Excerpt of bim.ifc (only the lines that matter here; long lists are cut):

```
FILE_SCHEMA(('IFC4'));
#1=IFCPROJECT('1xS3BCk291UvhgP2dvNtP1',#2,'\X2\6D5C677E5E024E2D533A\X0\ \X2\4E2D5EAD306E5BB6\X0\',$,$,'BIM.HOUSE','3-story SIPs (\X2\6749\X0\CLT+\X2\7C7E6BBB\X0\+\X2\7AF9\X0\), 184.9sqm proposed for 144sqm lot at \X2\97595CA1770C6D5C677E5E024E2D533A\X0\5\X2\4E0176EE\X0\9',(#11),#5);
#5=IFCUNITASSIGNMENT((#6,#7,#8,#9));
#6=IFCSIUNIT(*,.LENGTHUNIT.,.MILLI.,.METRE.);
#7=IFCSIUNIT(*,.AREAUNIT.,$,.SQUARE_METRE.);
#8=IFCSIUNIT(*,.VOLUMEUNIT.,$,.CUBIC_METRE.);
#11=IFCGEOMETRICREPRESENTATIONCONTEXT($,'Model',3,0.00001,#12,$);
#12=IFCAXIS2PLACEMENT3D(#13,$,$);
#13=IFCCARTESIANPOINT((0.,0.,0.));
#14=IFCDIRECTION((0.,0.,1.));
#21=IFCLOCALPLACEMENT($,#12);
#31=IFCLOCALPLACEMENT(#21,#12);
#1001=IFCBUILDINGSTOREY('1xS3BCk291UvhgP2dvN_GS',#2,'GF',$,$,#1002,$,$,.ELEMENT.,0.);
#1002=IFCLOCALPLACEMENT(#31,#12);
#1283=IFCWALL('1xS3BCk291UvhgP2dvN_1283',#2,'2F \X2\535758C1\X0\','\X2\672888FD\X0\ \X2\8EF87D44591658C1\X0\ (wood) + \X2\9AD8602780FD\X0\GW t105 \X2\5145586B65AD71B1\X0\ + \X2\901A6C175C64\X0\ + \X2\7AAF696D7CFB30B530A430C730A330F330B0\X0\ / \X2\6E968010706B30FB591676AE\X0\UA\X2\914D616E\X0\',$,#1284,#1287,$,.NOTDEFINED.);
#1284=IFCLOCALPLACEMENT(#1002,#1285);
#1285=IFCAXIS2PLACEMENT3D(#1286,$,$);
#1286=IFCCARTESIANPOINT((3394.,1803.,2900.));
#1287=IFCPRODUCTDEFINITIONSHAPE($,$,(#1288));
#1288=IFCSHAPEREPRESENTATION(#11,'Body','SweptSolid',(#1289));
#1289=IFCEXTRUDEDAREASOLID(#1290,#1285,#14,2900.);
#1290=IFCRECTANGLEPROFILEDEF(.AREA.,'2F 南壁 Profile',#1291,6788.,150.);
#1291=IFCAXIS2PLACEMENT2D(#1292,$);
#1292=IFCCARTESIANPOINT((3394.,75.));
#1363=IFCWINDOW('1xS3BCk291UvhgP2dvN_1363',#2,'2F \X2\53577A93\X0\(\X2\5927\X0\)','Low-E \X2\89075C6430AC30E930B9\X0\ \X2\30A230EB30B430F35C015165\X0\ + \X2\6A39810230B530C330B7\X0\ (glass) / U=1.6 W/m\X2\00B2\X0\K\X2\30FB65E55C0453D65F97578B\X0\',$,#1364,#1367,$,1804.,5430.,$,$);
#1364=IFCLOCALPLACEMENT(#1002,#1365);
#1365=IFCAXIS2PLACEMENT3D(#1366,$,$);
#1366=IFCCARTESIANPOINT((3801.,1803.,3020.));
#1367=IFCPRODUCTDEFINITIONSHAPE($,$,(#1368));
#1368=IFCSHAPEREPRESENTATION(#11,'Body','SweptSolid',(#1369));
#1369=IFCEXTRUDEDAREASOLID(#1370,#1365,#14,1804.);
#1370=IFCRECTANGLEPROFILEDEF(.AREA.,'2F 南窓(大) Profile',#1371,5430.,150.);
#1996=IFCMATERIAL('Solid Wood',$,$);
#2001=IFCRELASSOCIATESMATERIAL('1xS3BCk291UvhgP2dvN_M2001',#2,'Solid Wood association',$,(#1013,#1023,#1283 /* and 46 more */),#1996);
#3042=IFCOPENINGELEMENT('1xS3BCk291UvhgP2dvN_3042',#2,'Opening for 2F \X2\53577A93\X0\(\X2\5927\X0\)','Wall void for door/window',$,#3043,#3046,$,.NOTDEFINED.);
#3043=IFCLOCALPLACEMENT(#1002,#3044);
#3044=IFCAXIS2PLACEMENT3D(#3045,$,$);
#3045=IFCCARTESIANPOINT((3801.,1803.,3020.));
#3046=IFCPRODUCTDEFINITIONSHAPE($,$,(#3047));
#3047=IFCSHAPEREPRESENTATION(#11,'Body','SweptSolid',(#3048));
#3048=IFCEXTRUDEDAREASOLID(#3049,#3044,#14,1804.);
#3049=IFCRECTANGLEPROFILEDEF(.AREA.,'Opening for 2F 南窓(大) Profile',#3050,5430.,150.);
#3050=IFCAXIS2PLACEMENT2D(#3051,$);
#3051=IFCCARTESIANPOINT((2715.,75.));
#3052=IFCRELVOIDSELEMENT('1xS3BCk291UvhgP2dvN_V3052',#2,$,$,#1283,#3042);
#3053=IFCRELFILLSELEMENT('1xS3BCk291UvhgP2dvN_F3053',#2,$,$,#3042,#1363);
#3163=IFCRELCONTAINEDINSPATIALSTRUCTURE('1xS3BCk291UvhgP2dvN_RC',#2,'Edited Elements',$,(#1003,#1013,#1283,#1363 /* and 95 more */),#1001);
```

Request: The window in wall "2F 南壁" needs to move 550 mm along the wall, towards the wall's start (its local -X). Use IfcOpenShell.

```python
import ifcopenshell
import ifcopenshell.api.geometry
import ifcopenshell.util.placement
import ifcopenshell.util.unit

model = ifcopenshell.open("bim.ifc")
unit_scale = ifcopenshell.util.unit.calculate_unit_scale(model)

window = model.by_guid("1xS3BCk291UvhgP2dvN_1363")
opening = window.FillsVoids[0].RelatingOpeningElement
wall = opening.VoidsElements[0].RelatingBuildingElement

wall_matrix = ifcopenshell.util.placement.get_local_placement(wall.ObjectPlacement)
shift = wall_matrix[:3, 0] * -0.55 / unit_scale
before = ifcopenshell.util.placement.get_local_placement(window.ObjectPlacement)[:3, 3].copy()

# The window is not placed relative to its opening, so move both.
for product in (opening, window):
    matrix = ifcopenshell.util.placement.get_local_placement(product.ObjectPlacement)
    matrix[:3, 3] += shift
    ifcopenshell.api.geometry.edit_object_placement(model, product=product, matrix=matrix, is_si=False)

after = ifcopenshell.util.placement.get_local_placement(window.ObjectPlacement)[:3, 3]
print("window moved by", (after - before).round(3) + 0.0)

model.write("bim_updated.ifc")
```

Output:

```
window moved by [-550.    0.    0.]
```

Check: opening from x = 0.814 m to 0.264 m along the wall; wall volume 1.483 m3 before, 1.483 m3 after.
